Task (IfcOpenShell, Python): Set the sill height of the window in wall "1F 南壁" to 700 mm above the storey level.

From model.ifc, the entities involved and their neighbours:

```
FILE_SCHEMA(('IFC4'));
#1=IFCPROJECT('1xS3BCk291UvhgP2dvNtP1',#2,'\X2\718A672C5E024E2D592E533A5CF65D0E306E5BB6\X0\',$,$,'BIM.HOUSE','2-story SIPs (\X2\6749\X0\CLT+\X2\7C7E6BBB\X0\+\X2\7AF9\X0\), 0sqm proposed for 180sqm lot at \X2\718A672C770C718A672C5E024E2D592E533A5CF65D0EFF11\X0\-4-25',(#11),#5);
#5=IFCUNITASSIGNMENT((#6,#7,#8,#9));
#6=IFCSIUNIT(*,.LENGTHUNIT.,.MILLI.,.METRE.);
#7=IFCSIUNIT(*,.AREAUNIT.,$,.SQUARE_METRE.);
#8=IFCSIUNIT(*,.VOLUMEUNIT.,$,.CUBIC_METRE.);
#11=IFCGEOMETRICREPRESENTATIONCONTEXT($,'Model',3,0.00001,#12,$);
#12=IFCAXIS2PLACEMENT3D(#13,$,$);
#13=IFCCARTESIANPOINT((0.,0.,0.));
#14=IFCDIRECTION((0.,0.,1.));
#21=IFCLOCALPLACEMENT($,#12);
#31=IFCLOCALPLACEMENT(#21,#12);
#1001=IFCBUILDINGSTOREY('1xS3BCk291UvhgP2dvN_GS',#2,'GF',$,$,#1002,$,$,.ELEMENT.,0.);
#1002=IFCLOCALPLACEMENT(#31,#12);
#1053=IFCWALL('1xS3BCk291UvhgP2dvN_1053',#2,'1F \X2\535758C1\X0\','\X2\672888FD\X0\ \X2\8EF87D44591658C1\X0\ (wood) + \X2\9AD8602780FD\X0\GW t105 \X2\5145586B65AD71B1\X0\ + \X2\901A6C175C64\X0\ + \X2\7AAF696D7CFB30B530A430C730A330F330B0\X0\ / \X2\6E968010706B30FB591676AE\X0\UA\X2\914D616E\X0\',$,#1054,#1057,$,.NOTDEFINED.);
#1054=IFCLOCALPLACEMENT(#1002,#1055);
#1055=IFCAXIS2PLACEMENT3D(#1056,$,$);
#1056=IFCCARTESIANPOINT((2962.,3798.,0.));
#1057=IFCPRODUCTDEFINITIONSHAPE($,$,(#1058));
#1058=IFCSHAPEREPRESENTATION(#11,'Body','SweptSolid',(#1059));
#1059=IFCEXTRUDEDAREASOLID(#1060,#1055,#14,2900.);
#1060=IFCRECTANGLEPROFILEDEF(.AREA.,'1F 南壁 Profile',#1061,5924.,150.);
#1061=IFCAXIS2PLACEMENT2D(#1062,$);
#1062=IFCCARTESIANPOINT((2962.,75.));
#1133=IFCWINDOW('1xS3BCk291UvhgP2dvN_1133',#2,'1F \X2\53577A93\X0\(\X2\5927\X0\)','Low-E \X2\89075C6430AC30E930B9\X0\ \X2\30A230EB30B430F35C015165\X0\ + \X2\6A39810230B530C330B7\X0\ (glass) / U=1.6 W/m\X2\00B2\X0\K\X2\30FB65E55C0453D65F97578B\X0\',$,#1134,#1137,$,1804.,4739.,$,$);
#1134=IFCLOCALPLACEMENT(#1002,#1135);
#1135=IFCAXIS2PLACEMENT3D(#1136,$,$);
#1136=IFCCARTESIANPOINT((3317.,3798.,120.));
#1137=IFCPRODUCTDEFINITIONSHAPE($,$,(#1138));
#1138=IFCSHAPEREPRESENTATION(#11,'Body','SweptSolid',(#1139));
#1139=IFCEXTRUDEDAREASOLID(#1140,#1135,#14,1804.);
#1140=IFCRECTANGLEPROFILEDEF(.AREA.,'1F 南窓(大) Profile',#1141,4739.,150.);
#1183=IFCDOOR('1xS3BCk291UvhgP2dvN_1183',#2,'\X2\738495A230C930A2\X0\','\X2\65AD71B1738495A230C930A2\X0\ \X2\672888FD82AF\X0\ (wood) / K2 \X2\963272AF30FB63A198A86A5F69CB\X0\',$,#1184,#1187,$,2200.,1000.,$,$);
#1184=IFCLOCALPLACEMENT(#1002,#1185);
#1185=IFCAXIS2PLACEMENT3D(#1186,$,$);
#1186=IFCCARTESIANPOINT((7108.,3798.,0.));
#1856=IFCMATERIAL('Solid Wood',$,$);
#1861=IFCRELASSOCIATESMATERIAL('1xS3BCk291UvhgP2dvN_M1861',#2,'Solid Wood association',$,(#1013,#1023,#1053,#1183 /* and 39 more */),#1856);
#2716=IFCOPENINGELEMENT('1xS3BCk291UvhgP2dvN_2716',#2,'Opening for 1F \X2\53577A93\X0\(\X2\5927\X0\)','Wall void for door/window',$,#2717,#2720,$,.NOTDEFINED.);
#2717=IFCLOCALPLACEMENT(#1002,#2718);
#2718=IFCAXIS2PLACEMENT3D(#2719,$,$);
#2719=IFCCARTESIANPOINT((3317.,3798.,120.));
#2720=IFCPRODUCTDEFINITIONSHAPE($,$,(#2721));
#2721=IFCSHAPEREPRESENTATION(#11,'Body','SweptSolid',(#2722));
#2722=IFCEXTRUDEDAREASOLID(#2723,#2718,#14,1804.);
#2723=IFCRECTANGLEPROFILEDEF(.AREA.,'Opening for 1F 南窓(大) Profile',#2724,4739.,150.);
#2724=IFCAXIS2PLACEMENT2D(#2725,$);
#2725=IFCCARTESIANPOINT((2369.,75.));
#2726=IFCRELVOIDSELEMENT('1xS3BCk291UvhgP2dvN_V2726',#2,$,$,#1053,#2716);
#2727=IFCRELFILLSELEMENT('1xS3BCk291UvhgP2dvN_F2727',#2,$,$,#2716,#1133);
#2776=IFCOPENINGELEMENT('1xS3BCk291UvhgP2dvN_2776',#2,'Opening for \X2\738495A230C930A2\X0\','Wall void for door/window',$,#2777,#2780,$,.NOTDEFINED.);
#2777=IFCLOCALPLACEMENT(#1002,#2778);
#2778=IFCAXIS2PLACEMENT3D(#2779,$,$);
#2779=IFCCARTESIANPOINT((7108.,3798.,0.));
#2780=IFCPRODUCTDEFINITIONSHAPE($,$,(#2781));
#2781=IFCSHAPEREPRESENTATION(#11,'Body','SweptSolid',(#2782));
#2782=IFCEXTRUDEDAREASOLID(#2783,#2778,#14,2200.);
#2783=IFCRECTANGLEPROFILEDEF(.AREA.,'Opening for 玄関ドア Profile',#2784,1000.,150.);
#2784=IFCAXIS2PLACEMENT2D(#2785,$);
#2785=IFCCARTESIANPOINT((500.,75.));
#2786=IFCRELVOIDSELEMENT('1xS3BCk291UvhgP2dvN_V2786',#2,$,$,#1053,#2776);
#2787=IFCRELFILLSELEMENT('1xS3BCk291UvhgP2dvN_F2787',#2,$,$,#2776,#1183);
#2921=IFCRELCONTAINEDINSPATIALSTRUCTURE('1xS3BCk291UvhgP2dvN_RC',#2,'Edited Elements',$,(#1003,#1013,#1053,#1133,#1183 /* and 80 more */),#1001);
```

```python
import numpy as np
import ifcopenshell
import ifcopenshell.api.geometry
import ifcopenshell.geom
import ifcopenshell.util.element
import ifcopenshell.util.placement
import ifcopenshell.util.shape
import ifcopenshell.util.unit

model = ifcopenshell.open("model.ifc")
unit_scale = ifcopenshell.util.unit.calculate_unit_scale(model)

window = model.by_id(1133)
opening = window.FillsVoids[0].RelatingOpeningElement
storey = ifcopenshell.util.element.get_container(window, ifc_class="IfcBuildingStorey")
level = ifcopenshell.util.placement.get_local_placement(storey.ObjectPlacement)[2, 3]

# The opening's origin need not be at the sill, so measure its lowest point.
shape = ifcopenshell.geom.create_shape(ifcopenshell.geom.settings(), opening)
bottom = ifcopenshell.util.shape.get_shape_bottom_elevation(shape, shape.geometry) / unit_scale
dz = level + 0.7 / unit_scale - bottom

shift = np.array([0.0, 0.0, dz])
# The window is not placed relative to its opening, so move both.
for product in (opening, window):
    matrix = ifcopenshell.util.placement.get_local_placement(product.ObjectPlacement)
    matrix[:3, 3] += shift
    ifcopenshell.api.geometry.edit_object_placement(model, product=product, matrix=matrix, is_si=False)

print(f"moved by {dz * unit_scale:+.3f} m")

model.write("model_rev.ifc")
```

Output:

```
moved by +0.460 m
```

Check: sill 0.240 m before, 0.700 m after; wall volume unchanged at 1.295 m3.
